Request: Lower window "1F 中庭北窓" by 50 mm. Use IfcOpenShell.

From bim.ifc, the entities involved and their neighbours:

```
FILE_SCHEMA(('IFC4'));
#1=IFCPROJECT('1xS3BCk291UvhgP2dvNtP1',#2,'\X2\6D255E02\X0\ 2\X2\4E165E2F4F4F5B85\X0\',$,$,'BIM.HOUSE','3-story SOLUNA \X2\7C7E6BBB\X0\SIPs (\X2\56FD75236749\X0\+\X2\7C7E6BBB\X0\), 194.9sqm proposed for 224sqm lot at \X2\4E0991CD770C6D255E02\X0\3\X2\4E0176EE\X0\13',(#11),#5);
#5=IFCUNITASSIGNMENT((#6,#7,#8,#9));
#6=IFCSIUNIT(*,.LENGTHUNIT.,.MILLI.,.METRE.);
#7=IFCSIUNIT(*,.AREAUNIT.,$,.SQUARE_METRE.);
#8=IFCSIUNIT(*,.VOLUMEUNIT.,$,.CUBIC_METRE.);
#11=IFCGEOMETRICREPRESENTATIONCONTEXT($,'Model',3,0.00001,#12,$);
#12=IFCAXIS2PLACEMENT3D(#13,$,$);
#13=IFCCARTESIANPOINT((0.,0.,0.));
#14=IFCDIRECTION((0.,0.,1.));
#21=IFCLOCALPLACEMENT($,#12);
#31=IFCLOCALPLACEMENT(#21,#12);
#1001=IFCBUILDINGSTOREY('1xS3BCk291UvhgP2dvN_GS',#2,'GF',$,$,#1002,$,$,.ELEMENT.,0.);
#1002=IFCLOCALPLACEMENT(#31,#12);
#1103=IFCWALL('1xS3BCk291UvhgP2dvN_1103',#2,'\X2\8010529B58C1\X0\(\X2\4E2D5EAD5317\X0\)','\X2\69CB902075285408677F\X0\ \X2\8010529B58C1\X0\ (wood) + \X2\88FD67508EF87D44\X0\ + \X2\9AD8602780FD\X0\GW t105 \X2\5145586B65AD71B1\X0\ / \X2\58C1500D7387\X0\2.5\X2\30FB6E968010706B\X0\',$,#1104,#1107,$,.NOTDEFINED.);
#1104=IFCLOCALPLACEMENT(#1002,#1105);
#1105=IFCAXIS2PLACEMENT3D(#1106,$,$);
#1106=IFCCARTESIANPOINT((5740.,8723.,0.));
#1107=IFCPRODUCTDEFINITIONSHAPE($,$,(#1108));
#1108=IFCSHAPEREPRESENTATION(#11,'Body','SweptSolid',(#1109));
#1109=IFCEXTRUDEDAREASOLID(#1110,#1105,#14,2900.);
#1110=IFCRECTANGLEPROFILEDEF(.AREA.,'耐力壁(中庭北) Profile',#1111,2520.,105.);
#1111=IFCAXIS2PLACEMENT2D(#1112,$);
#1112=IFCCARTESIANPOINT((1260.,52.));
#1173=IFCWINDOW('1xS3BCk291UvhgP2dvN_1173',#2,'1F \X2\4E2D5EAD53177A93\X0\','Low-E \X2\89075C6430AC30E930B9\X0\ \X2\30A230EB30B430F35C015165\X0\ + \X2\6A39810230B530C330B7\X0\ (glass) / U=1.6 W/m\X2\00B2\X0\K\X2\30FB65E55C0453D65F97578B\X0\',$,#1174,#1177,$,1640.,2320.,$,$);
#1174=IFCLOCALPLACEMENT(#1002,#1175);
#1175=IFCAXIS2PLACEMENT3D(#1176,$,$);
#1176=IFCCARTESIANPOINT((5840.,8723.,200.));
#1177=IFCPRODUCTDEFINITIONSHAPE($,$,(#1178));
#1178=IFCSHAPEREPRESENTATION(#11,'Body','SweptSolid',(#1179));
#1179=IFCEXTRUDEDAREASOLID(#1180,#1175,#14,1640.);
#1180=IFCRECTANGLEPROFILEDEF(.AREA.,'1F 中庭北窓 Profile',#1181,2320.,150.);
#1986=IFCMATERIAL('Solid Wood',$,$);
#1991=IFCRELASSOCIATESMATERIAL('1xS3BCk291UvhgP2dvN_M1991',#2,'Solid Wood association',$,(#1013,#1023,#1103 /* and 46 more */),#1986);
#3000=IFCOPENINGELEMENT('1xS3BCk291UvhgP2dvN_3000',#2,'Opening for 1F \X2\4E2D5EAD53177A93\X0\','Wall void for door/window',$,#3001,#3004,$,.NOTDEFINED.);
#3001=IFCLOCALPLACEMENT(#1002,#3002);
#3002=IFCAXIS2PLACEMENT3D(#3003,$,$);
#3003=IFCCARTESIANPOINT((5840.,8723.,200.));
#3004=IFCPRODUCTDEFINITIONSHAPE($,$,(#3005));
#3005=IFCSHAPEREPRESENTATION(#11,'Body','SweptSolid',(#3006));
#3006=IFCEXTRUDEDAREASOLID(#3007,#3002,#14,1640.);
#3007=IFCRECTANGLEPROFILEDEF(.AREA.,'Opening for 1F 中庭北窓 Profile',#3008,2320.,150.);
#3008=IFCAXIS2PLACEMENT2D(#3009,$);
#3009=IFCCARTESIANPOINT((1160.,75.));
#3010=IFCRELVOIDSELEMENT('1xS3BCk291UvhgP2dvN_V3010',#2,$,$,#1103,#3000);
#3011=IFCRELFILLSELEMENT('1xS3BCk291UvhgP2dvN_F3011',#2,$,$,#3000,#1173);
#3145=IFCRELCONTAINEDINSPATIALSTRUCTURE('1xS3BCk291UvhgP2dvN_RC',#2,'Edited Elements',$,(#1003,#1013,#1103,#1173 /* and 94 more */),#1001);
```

```python
import numpy as np
import ifcopenshell
import ifcopenshell.api.geometry
import ifcopenshell.util.placement
import ifcopenshell.util.unit

model = ifcopenshell.open("bim.ifc")
unit_scale = ifcopenshell.util.unit.calculate_unit_scale(model)

window = model.by_id(1173)
opening = window.FillsVoids[0].RelatingOpeningElement
dz = -50.0

shift = np.array([0.0, 0.0, dz])
# The window is not placed relative to its opening, so move both.
for product in (opening, window):
    matrix = ifcopenshell.util.placement.get_local_placement(product.ObjectPlacement)
    matrix[:3, 3] += shift
    ifcopenshell.api.geometry.edit_object_placement(model, product=product, matrix=matrix, is_si=False)

print(f"moved by {dz * unit_scale:+.3f} m")

model.write("bim-out.ifc")
```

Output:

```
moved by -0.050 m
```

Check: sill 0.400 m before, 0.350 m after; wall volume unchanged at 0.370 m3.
